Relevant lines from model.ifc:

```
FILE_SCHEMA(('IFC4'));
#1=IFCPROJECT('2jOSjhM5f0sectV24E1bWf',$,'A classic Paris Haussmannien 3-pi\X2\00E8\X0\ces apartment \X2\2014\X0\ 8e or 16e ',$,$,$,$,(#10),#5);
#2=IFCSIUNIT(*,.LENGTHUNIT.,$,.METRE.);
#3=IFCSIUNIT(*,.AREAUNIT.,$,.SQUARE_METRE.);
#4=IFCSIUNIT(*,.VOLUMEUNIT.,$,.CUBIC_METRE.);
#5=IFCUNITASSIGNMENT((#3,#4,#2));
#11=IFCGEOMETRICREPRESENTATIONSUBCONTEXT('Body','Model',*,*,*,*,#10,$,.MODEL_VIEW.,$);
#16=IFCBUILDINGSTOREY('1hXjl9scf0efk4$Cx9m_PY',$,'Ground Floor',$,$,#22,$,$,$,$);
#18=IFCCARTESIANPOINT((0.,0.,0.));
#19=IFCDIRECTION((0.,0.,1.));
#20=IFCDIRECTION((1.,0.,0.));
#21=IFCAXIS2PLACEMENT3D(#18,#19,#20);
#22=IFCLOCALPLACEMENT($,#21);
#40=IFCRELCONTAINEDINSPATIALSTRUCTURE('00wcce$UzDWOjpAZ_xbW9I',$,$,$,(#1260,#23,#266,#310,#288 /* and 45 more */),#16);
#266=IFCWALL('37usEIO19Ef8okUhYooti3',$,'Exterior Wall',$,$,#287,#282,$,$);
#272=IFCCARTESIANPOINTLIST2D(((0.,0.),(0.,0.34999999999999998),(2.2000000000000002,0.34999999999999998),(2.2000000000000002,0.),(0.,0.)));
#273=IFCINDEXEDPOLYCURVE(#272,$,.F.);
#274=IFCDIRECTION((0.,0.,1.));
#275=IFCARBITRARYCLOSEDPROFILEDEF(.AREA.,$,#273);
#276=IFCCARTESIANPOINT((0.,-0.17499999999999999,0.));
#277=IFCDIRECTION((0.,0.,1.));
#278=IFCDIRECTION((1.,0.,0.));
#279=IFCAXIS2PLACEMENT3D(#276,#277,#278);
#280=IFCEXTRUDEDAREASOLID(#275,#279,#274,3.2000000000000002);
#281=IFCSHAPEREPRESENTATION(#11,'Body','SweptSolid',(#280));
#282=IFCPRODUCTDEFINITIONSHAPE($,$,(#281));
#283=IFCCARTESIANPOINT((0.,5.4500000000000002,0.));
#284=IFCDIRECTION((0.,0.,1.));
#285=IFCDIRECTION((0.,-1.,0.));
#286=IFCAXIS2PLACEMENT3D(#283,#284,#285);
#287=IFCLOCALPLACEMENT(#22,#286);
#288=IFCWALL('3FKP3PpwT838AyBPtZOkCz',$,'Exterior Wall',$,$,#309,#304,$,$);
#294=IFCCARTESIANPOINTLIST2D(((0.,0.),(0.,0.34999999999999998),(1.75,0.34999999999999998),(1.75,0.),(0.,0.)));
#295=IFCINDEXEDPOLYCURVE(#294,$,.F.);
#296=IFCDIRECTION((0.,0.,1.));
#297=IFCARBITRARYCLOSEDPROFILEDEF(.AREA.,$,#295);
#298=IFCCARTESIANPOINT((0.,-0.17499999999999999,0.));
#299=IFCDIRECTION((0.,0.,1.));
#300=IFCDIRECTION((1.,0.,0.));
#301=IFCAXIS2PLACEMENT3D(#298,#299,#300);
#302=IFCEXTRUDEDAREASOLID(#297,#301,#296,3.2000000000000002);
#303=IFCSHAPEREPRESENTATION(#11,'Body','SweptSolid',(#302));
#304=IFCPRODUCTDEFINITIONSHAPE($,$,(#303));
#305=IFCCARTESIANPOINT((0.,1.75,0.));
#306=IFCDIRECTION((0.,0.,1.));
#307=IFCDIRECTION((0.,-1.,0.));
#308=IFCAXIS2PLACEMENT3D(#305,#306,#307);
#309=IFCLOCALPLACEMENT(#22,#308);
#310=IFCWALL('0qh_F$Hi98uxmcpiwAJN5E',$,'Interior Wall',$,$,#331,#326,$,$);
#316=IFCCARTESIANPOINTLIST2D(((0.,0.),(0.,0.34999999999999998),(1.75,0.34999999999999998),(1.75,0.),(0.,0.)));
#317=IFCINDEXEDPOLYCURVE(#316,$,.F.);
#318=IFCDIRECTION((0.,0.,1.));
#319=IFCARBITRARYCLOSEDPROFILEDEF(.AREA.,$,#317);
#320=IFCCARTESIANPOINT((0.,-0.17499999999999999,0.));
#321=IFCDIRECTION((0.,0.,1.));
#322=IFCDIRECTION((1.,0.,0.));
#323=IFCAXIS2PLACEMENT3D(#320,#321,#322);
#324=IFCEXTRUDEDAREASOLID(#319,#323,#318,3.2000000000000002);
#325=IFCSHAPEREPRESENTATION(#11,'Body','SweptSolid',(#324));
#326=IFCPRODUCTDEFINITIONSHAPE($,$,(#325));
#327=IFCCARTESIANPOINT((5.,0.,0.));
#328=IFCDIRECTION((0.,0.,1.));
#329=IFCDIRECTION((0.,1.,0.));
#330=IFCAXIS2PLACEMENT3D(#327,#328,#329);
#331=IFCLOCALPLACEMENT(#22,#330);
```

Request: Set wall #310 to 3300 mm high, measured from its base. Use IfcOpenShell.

```python
import ifcopenshell
import ifcopenshell.geom
import ifcopenshell.util.representation
import ifcopenshell.util.shape

model = ifcopenshell.open("model.ifc")
settings = ifcopenshell.geom.settings()


def volume(element):
    """Net volume in cubic metres, openings subtracted."""
    shape = ifcopenshell.geom.create_shape(settings, element)
    return ifcopenshell.util.shape.get_volume(shape.geometry)


wall = model.by_id(310)
before = volume(wall)

body = ifcopenshell.util.representation.get_representation(wall, "Model", "Body")
solid = body.Items[0]
old_height = solid.Depth
solid.Depth = 3.3
after = volume(wall)

print(f"height {old_height:g} -> {solid.Depth:g}, volume {before:.3f} -> {after:.3f} m3")

model.write("model-out.ifc")
```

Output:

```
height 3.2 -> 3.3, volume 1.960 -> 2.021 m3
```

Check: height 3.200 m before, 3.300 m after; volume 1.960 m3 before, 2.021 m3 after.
